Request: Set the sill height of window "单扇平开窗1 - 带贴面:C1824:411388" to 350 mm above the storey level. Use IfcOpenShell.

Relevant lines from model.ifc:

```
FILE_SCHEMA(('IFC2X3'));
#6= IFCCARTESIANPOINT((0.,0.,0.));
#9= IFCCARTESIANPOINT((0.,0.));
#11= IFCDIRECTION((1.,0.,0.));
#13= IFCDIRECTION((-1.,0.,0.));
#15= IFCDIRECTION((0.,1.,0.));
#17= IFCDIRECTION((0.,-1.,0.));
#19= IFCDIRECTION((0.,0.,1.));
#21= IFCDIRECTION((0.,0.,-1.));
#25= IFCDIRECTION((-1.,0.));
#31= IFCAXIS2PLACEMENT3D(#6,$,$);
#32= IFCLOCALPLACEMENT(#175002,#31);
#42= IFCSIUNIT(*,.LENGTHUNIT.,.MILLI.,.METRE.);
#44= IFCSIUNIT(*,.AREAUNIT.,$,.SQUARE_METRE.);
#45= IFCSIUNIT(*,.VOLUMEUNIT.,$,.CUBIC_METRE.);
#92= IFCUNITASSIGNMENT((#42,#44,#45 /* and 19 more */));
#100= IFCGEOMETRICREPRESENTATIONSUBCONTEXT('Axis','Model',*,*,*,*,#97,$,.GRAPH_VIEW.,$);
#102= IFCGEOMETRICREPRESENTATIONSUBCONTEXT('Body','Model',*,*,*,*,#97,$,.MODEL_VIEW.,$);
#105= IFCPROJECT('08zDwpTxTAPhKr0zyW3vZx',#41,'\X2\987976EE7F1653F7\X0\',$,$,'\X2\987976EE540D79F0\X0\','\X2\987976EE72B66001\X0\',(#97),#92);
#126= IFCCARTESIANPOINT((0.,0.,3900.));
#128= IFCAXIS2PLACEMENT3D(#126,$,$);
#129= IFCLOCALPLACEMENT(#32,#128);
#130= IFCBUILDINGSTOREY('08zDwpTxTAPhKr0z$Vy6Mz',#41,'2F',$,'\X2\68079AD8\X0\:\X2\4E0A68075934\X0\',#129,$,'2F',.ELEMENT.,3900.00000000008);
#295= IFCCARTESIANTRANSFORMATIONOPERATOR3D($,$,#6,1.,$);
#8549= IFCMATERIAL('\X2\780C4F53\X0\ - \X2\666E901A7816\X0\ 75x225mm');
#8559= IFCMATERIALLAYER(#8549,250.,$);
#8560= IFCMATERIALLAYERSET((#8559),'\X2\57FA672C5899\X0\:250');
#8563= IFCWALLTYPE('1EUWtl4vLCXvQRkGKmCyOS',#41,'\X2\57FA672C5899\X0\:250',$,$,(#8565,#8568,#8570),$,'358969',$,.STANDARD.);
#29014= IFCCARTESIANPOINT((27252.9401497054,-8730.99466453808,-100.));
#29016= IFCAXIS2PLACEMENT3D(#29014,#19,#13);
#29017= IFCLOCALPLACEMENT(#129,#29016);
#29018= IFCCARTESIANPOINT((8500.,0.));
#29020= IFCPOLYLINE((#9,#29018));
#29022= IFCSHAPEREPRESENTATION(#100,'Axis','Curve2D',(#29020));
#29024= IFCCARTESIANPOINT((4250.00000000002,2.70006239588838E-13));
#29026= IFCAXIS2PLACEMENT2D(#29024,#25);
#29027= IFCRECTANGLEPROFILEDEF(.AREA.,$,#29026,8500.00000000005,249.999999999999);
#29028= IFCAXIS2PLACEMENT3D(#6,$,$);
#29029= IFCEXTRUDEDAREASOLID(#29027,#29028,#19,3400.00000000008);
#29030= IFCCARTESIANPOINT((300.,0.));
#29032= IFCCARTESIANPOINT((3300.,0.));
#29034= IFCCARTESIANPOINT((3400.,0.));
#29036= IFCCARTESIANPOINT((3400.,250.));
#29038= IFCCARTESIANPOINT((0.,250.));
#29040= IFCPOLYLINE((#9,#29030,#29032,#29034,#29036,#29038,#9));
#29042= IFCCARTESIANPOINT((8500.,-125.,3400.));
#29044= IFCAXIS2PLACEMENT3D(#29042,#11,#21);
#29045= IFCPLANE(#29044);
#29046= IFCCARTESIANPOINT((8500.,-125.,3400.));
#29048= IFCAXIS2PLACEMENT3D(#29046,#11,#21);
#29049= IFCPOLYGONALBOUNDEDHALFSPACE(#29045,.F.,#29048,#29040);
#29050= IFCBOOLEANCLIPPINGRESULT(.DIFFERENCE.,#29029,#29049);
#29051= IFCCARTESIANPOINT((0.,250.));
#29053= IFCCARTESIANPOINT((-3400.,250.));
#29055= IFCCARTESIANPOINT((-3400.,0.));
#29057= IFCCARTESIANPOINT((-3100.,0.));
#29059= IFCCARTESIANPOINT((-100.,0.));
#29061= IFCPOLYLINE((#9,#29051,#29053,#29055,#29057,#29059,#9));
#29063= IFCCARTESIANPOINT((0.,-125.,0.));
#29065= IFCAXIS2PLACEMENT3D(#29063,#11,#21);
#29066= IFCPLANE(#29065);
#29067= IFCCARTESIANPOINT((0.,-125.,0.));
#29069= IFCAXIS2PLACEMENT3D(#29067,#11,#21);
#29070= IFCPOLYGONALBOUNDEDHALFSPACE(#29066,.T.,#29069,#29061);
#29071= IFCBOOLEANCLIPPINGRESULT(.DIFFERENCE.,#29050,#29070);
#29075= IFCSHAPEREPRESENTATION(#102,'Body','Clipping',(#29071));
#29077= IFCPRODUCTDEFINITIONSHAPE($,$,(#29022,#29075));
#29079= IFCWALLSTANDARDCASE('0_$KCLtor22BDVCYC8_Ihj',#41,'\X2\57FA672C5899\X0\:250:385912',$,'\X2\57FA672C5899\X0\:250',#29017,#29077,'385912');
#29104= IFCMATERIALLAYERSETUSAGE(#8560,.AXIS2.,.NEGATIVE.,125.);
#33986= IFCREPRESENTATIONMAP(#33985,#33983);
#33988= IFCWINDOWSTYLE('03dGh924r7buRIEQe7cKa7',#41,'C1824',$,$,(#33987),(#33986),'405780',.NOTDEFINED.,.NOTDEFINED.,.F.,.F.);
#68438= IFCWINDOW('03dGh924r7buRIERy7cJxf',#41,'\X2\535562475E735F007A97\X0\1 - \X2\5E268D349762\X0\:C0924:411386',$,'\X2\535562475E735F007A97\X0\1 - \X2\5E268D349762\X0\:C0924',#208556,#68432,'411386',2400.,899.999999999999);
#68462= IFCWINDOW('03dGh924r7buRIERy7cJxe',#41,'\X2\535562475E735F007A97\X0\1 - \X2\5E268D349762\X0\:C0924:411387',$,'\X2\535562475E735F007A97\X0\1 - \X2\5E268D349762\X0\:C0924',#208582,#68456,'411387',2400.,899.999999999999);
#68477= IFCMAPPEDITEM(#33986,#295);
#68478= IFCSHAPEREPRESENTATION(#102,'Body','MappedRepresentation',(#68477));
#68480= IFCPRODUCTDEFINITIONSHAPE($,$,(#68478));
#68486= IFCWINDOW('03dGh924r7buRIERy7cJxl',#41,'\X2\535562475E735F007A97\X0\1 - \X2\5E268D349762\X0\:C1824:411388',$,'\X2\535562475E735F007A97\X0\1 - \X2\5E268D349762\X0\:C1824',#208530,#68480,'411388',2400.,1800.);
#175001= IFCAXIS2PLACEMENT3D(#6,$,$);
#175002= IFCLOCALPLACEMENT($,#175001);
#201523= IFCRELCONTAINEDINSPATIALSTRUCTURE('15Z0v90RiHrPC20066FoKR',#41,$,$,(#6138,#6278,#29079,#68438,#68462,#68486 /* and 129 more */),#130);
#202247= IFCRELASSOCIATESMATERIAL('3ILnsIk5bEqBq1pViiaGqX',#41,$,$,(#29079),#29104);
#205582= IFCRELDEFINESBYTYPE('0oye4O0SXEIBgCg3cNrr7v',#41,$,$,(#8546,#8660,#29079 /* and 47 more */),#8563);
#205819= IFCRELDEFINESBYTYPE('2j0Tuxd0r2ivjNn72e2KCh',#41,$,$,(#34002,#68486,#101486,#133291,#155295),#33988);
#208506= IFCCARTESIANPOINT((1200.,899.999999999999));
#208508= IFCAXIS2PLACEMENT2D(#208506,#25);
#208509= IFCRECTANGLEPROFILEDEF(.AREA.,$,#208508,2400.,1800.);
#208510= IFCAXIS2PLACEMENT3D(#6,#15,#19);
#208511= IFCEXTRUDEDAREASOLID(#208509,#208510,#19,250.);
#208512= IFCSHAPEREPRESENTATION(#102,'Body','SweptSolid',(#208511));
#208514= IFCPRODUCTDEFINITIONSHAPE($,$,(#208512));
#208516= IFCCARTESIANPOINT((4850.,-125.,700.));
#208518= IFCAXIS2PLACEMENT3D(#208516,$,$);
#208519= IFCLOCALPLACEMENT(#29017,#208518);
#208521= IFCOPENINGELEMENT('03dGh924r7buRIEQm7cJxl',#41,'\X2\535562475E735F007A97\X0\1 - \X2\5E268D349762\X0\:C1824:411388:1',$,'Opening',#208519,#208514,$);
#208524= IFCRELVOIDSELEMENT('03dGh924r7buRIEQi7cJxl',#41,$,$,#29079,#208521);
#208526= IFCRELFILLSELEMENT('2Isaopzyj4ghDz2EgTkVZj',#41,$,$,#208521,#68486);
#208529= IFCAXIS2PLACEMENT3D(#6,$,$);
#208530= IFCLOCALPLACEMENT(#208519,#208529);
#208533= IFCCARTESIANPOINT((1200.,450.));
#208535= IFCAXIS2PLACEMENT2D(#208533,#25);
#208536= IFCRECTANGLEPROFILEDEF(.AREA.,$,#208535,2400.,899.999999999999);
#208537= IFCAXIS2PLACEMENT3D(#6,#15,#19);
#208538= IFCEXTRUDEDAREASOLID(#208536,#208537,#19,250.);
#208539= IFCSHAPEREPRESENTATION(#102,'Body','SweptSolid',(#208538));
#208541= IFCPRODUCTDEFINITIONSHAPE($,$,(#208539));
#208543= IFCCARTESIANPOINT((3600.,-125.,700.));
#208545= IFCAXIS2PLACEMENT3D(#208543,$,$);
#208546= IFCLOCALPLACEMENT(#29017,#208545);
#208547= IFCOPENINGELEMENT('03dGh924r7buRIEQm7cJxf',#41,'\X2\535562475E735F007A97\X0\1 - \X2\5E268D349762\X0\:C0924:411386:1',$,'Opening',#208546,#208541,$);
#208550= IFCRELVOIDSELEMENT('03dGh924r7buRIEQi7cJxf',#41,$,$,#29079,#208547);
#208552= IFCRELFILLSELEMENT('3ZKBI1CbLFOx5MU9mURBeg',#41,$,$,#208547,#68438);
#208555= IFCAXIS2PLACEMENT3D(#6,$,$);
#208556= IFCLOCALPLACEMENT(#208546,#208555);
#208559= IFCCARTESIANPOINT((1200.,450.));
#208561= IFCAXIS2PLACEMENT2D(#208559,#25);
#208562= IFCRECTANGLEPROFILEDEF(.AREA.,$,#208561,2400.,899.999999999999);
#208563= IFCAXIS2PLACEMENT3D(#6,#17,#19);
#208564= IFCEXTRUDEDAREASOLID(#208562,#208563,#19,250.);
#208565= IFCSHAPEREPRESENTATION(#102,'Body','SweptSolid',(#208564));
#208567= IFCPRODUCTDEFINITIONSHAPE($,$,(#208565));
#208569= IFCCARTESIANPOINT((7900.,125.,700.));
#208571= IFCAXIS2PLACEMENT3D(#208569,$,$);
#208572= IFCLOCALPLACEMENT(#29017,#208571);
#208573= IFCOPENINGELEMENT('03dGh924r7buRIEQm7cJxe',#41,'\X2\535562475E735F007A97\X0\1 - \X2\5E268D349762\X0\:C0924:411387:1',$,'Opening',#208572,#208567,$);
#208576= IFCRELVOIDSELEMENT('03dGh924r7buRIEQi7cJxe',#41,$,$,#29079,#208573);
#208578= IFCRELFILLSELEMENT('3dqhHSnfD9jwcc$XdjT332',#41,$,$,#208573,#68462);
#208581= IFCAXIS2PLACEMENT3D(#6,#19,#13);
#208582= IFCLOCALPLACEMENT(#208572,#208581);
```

```python
import numpy as np
import ifcopenshell
import ifcopenshell.api.geometry
import ifcopenshell.geom
import ifcopenshell.util.element
import ifcopenshell.util.placement
import ifcopenshell.util.shape
import ifcopenshell.util.unit

model = ifcopenshell.open("model.ifc")
unit_scale = ifcopenshell.util.unit.calculate_unit_scale(model)

window = model.by_id(68486)
opening = window.FillsVoids[0].RelatingOpeningElement
storey = ifcopenshell.util.element.get_container(window, ifc_class="IfcBuildingStorey")
level = ifcopenshell.util.placement.get_local_placement(storey.ObjectPlacement)[2, 3]

# The opening's origin need not be at the sill, so measure its lowest point.
shape = ifcopenshell.geom.create_shape(ifcopenshell.geom.settings(), opening)
bottom = ifcopenshell.util.shape.get_shape_bottom_elevation(shape, shape.geometry) / unit_scale
dz = level + 350.0 - bottom

shift = np.array([0.0, 0.0, dz])
# The window is placed relative to its opening, so it follows when the opening moves.
matrix = ifcopenshell.util.placement.get_local_placement(opening.ObjectPlacement)
matrix[:3, 3] += shift
ifcopenshell.api.geometry.edit_object_placement(
    model, product=opening, matrix=matrix, is_si=False, should_transform_children=True
)

print(f"moved by {dz * unit_scale:+.3f} m")

model.write("model_updated.ifc")
```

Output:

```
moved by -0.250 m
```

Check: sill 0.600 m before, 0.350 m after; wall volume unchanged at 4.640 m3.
